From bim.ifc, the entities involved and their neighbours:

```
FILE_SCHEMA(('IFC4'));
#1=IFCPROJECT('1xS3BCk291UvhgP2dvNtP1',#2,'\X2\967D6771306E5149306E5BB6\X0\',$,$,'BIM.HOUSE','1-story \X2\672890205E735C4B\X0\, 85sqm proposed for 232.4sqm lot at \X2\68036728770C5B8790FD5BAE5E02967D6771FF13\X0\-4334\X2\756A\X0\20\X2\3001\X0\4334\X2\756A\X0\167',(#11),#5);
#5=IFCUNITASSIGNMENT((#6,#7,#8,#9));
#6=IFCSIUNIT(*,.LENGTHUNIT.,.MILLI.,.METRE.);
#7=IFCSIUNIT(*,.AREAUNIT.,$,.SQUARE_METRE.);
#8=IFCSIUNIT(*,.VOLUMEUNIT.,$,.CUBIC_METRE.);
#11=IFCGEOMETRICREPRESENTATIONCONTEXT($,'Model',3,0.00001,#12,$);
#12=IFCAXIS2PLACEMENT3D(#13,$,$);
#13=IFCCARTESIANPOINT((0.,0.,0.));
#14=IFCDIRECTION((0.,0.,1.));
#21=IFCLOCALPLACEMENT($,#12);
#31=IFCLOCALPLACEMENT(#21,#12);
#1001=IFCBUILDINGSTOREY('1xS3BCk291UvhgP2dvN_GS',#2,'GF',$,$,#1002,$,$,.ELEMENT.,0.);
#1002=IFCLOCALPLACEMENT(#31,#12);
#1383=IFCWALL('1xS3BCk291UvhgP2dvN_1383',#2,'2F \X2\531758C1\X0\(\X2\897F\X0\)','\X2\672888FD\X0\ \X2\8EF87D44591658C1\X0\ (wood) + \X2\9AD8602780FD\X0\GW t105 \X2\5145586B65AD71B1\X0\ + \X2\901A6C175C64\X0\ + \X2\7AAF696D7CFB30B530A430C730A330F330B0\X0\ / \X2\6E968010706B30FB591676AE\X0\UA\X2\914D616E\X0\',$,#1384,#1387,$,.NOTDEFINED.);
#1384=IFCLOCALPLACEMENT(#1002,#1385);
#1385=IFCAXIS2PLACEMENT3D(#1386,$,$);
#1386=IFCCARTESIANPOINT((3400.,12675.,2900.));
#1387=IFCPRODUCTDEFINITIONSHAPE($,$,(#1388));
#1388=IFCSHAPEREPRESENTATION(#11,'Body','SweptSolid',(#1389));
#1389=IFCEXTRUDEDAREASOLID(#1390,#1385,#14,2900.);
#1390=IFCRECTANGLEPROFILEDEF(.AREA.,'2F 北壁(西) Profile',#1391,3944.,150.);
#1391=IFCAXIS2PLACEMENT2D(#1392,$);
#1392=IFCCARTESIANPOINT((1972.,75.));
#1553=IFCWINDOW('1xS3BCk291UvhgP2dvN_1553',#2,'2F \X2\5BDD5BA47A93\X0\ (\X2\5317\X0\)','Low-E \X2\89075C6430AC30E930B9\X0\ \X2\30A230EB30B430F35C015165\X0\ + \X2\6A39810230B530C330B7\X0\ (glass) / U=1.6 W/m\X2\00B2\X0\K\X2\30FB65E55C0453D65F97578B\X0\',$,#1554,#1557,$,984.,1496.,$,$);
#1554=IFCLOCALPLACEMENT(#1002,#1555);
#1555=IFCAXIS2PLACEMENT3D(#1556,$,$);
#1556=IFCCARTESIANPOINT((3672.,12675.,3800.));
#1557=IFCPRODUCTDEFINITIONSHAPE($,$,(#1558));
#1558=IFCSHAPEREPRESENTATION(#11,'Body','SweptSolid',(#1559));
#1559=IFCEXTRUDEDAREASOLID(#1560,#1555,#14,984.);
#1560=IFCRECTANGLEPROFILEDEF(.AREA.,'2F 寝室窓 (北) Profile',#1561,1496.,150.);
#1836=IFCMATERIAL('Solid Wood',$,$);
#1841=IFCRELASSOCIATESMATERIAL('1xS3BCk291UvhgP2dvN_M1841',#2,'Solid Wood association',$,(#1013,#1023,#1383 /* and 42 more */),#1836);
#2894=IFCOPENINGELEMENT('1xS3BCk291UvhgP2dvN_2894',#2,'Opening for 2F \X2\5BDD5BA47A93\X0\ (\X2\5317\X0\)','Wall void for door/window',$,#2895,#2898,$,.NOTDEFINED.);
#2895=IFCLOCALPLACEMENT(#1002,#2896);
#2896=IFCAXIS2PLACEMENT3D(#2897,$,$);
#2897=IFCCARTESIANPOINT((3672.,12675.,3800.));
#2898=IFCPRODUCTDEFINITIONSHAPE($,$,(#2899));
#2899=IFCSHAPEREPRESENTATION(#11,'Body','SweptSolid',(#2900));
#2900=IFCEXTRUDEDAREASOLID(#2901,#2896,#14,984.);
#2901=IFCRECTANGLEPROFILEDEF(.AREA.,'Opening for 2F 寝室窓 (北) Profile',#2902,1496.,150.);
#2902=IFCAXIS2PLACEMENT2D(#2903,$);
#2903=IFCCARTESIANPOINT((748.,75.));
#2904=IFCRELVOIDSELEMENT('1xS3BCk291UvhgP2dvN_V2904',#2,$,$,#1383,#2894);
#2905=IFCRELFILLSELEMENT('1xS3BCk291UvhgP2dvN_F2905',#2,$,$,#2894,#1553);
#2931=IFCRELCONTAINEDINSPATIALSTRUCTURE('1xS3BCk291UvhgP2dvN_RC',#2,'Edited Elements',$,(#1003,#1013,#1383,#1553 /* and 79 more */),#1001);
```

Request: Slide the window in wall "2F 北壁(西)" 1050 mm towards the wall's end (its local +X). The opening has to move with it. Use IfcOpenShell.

```python
import ifcopenshell
import ifcopenshell.api.geometry
import ifcopenshell.util.placement
import ifcopenshell.util.unit

model = ifcopenshell.open("bim.ifc")
unit_scale = ifcopenshell.util.unit.calculate_unit_scale(model)

window = model.by_guid("1xS3BCk291UvhgP2dvN_1553")
opening = window.FillsVoids[0].RelatingOpeningElement
wall = opening.VoidsElements[0].RelatingBuildingElement

wall_matrix = ifcopenshell.util.placement.get_local_placement(wall.ObjectPlacement)
shift = wall_matrix[:3, 0] * 1.05 / unit_scale
before = ifcopenshell.util.placement.get_local_placement(window.ObjectPlacement)[:3, 3].copy()

# The window is not placed relative to its opening, so move both.
for product in (opening, window):
    matrix = ifcopenshell.util.placement.get_local_placement(product.ObjectPlacement)
    matrix[:3, 3] += shift
    ifcopenshell.api.geometry.edit_object_placement(model, product=product, matrix=matrix, is_si=False)

after = ifcopenshell.util.placement.get_local_placement(window.ObjectPlacement)[:3, 3]
print("window moved by", (after - before).round(3) + 0.0)

model.write("bim_updated.ifc")
```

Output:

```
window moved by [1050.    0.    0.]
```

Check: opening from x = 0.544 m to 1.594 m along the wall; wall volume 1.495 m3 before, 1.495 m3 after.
